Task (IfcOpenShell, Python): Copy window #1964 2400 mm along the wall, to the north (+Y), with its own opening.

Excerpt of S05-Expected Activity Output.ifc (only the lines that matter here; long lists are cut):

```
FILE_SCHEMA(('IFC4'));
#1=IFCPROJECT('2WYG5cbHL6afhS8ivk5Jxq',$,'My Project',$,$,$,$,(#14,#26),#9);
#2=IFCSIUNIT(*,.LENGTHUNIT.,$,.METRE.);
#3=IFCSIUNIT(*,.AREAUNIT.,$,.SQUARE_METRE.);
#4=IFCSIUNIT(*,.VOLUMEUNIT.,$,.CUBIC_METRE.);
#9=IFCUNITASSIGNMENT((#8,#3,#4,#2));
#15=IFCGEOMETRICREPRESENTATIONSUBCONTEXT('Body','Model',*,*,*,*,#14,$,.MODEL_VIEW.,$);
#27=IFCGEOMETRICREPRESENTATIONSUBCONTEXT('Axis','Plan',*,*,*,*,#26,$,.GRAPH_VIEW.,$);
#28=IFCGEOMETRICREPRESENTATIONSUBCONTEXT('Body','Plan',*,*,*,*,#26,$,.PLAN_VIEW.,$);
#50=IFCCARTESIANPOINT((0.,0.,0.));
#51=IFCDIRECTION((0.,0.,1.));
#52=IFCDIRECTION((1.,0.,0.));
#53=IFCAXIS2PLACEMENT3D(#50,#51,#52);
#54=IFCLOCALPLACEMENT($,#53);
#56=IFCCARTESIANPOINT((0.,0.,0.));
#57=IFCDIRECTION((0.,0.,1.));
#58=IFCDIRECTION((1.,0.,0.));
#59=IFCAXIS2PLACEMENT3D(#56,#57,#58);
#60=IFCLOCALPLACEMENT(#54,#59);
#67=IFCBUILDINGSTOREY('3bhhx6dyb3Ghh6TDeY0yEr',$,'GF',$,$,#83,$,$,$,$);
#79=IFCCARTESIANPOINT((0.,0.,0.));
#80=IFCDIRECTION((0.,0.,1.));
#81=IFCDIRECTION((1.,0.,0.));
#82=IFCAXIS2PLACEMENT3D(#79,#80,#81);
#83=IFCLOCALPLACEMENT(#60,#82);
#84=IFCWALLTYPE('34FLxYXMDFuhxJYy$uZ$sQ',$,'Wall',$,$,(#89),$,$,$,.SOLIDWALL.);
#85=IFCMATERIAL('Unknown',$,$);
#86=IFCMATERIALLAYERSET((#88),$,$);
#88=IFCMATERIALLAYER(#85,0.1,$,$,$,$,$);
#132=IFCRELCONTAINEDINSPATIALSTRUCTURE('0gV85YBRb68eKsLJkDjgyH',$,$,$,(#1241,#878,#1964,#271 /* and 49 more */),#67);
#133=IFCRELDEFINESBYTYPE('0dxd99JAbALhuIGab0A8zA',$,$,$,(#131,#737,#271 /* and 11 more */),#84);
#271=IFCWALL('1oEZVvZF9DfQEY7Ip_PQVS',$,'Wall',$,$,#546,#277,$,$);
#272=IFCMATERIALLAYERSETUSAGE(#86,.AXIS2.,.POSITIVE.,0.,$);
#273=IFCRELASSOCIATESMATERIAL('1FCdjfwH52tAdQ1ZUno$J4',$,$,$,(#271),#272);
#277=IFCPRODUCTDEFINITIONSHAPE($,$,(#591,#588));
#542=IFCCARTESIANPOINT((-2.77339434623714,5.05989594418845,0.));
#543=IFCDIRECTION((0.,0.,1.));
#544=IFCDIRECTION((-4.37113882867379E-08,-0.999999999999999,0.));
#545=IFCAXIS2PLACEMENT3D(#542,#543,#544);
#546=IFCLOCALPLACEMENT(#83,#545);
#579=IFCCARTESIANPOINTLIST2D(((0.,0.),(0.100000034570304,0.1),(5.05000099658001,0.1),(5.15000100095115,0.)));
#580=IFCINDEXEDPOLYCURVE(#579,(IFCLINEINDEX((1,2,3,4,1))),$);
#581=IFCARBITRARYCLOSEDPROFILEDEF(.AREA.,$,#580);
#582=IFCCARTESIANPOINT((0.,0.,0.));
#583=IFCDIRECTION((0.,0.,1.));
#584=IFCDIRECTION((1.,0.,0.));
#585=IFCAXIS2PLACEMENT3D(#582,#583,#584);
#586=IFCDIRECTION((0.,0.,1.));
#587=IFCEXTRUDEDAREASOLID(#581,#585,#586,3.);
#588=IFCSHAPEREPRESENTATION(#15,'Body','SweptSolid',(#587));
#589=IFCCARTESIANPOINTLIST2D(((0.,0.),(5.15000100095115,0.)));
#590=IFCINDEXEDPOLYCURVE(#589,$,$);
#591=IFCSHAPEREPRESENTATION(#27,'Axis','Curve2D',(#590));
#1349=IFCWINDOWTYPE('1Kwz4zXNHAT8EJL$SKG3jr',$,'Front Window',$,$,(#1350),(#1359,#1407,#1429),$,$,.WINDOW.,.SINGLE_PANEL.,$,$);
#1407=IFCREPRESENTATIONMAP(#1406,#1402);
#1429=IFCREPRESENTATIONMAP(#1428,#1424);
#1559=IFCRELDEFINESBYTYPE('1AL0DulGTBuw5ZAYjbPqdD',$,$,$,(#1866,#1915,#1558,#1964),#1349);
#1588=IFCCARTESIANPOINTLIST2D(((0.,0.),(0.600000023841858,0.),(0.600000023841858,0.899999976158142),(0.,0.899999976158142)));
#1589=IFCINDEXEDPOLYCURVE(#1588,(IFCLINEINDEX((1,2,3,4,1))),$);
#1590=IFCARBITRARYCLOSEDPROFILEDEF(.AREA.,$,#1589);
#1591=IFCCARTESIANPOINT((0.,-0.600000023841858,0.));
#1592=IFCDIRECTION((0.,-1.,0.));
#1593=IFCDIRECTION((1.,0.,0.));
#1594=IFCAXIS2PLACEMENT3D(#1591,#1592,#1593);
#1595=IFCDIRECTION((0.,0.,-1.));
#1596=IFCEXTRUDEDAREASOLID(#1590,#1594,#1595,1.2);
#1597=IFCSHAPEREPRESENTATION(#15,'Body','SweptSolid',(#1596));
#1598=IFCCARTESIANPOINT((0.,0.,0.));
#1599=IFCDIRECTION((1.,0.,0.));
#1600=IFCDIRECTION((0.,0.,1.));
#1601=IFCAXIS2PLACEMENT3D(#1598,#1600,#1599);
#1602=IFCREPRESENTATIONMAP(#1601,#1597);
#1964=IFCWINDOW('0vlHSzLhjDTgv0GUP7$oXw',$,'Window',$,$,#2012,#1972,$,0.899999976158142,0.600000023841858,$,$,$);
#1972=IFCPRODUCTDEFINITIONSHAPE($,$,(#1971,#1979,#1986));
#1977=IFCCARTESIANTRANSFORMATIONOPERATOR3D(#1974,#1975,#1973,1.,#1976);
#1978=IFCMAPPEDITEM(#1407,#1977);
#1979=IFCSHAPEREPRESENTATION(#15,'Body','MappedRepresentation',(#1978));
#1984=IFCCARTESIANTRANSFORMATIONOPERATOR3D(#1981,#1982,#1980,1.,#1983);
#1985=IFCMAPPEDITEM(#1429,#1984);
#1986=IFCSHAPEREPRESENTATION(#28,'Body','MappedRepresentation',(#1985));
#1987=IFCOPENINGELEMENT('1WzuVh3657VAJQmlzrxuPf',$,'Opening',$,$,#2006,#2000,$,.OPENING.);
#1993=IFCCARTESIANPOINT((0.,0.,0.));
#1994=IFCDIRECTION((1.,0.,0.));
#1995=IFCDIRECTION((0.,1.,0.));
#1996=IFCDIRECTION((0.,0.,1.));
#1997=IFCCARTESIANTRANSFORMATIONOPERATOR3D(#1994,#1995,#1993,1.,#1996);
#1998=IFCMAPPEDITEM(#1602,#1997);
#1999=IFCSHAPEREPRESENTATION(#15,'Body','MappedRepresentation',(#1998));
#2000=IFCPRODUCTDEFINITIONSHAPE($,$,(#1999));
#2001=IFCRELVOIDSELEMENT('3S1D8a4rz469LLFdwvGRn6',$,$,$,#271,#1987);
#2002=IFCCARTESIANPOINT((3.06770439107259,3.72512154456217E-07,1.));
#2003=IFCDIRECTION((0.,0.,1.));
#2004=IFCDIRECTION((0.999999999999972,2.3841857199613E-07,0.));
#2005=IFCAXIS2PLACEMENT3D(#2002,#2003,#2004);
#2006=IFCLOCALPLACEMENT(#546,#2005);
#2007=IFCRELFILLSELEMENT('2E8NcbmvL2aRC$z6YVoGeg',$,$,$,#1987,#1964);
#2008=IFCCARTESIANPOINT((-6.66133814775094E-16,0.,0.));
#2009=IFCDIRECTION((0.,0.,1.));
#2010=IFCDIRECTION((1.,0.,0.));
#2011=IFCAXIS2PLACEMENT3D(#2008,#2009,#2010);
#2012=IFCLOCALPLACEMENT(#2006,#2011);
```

```python
import ifcopenshell
import ifcopenshell.api.feature
import ifcopenshell.api.geometry
import ifcopenshell.api.root
import ifcopenshell.geom
import ifcopenshell.util.element
import ifcopenshell.util.placement
import ifcopenshell.util.shape
import ifcopenshell.util.unit

model = ifcopenshell.open("S05-Expected Activity Output.ifc")
unit_scale = ifcopenshell.util.unit.calculate_unit_scale(model)
settings = ifcopenshell.geom.settings()


def volume(element):
    """Net volume in cubic metres, openings subtracted."""
    shape = ifcopenshell.geom.create_shape(settings, element)
    return ifcopenshell.util.shape.get_volume(shape.geometry)


window = model.by_guid("0vlHSzLhjDTgv0GUP7$oXw")
opening = window.FillsVoids[0].RelatingOpeningElement
wall = opening.VoidsElements[0].RelatingBuildingElement
before = volume(wall)
shift = ifcopenshell.util.placement.get_local_placement(wall.ObjectPlacement)[:3, 0] * -2.4 / unit_scale

# copy_class copies the void relationship, type, container and properties, but no geometry.
new_opening = ifcopenshell.api.root.copy_class(model, product=opening)
new_opening.Representation = ifcopenshell.util.element.copy_deep(
    model, opening.Representation, exclude=["IfcGeometricRepresentationContext", "IfcRepresentationMap"]
)
new_window = ifcopenshell.api.root.copy_class(model, product=window)
new_window.Representation = ifcopenshell.util.element.copy_deep(
    model, window.Representation, exclude=["IfcGeometricRepresentationContext", "IfcRepresentationMap"]
)
ifcopenshell.api.feature.add_filling(model, opening=new_opening, element=new_window)

for old, new in ((opening, new_opening), (window, new_window)):
    matrix = ifcopenshell.util.placement.get_local_placement(old.ObjectPlacement)
    matrix[:3, 3] += shift
    ifcopenshell.api.geometry.edit_object_placement(model, product=new, matrix=matrix, is_si=False)

after = volume(wall)

print(f"wall volume {before:.3f} -> {after:.3f} m3")

model.write("S05-Expected Activity Output_updated.ifc")
```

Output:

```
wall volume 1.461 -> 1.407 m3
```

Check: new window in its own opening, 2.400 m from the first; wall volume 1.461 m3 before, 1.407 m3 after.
